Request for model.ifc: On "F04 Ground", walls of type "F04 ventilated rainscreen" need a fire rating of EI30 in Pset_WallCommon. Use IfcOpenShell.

First a look at what the model holds.

```python
import ifcopenshell
import ifcopenshell.util.element

model = ifcopenshell.open("model.ifc")
print(model.schema)
storey = next(s for s in model.by_type("IfcBuildingStorey") if s.Name == "F04 Ground")
walls = [e for e in ifcopenshell.util.element.get_decomposition(storey) if e.is_a("IfcWall")]
seen = {}
for e in walls:
    element_type = ifcopenshell.util.element.get_type(e)
    key = (element_type.Name if element_type != e and element_type else None, ifcopenshell.util.element.get_pset(e, "Pset_WallCommon", "FireRating"))
    seen[key] = seen.get(key, 0) + 1
for (name, value), count in sorted(seen.items(), key=str):
    print(count, "x", name, "|", value)
```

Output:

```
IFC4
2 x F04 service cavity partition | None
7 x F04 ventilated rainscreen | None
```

```python
import ifcopenshell
import ifcopenshell.api.pset
import ifcopenshell.util.element

model = ifcopenshell.open("model.ifc")

storey = next(s for s in model.by_type("IfcBuildingStorey") if s.Name == "F04 Ground")
walls = [e for e in ifcopenshell.util.element.get_decomposition(storey) if e.is_a("IfcWall")]

count = 0
for e in walls:
    element_type = ifcopenshell.util.element.get_type(e)
    if element_type in (None, e) or element_type.Name != "F04 ventilated rainscreen":
        continue
    # add_pset returns the element's existing set when there is one.
    pset = ifcopenshell.api.pset.add_pset(model, product=e, name="Pset_WallCommon")
    ifcopenshell.api.pset.edit_pset(model, pset=pset, properties={"FireRating": "EI30"})
    count += 1

print(count, "walls updated")

model.write("model-out.ifc")
```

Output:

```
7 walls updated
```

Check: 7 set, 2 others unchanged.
